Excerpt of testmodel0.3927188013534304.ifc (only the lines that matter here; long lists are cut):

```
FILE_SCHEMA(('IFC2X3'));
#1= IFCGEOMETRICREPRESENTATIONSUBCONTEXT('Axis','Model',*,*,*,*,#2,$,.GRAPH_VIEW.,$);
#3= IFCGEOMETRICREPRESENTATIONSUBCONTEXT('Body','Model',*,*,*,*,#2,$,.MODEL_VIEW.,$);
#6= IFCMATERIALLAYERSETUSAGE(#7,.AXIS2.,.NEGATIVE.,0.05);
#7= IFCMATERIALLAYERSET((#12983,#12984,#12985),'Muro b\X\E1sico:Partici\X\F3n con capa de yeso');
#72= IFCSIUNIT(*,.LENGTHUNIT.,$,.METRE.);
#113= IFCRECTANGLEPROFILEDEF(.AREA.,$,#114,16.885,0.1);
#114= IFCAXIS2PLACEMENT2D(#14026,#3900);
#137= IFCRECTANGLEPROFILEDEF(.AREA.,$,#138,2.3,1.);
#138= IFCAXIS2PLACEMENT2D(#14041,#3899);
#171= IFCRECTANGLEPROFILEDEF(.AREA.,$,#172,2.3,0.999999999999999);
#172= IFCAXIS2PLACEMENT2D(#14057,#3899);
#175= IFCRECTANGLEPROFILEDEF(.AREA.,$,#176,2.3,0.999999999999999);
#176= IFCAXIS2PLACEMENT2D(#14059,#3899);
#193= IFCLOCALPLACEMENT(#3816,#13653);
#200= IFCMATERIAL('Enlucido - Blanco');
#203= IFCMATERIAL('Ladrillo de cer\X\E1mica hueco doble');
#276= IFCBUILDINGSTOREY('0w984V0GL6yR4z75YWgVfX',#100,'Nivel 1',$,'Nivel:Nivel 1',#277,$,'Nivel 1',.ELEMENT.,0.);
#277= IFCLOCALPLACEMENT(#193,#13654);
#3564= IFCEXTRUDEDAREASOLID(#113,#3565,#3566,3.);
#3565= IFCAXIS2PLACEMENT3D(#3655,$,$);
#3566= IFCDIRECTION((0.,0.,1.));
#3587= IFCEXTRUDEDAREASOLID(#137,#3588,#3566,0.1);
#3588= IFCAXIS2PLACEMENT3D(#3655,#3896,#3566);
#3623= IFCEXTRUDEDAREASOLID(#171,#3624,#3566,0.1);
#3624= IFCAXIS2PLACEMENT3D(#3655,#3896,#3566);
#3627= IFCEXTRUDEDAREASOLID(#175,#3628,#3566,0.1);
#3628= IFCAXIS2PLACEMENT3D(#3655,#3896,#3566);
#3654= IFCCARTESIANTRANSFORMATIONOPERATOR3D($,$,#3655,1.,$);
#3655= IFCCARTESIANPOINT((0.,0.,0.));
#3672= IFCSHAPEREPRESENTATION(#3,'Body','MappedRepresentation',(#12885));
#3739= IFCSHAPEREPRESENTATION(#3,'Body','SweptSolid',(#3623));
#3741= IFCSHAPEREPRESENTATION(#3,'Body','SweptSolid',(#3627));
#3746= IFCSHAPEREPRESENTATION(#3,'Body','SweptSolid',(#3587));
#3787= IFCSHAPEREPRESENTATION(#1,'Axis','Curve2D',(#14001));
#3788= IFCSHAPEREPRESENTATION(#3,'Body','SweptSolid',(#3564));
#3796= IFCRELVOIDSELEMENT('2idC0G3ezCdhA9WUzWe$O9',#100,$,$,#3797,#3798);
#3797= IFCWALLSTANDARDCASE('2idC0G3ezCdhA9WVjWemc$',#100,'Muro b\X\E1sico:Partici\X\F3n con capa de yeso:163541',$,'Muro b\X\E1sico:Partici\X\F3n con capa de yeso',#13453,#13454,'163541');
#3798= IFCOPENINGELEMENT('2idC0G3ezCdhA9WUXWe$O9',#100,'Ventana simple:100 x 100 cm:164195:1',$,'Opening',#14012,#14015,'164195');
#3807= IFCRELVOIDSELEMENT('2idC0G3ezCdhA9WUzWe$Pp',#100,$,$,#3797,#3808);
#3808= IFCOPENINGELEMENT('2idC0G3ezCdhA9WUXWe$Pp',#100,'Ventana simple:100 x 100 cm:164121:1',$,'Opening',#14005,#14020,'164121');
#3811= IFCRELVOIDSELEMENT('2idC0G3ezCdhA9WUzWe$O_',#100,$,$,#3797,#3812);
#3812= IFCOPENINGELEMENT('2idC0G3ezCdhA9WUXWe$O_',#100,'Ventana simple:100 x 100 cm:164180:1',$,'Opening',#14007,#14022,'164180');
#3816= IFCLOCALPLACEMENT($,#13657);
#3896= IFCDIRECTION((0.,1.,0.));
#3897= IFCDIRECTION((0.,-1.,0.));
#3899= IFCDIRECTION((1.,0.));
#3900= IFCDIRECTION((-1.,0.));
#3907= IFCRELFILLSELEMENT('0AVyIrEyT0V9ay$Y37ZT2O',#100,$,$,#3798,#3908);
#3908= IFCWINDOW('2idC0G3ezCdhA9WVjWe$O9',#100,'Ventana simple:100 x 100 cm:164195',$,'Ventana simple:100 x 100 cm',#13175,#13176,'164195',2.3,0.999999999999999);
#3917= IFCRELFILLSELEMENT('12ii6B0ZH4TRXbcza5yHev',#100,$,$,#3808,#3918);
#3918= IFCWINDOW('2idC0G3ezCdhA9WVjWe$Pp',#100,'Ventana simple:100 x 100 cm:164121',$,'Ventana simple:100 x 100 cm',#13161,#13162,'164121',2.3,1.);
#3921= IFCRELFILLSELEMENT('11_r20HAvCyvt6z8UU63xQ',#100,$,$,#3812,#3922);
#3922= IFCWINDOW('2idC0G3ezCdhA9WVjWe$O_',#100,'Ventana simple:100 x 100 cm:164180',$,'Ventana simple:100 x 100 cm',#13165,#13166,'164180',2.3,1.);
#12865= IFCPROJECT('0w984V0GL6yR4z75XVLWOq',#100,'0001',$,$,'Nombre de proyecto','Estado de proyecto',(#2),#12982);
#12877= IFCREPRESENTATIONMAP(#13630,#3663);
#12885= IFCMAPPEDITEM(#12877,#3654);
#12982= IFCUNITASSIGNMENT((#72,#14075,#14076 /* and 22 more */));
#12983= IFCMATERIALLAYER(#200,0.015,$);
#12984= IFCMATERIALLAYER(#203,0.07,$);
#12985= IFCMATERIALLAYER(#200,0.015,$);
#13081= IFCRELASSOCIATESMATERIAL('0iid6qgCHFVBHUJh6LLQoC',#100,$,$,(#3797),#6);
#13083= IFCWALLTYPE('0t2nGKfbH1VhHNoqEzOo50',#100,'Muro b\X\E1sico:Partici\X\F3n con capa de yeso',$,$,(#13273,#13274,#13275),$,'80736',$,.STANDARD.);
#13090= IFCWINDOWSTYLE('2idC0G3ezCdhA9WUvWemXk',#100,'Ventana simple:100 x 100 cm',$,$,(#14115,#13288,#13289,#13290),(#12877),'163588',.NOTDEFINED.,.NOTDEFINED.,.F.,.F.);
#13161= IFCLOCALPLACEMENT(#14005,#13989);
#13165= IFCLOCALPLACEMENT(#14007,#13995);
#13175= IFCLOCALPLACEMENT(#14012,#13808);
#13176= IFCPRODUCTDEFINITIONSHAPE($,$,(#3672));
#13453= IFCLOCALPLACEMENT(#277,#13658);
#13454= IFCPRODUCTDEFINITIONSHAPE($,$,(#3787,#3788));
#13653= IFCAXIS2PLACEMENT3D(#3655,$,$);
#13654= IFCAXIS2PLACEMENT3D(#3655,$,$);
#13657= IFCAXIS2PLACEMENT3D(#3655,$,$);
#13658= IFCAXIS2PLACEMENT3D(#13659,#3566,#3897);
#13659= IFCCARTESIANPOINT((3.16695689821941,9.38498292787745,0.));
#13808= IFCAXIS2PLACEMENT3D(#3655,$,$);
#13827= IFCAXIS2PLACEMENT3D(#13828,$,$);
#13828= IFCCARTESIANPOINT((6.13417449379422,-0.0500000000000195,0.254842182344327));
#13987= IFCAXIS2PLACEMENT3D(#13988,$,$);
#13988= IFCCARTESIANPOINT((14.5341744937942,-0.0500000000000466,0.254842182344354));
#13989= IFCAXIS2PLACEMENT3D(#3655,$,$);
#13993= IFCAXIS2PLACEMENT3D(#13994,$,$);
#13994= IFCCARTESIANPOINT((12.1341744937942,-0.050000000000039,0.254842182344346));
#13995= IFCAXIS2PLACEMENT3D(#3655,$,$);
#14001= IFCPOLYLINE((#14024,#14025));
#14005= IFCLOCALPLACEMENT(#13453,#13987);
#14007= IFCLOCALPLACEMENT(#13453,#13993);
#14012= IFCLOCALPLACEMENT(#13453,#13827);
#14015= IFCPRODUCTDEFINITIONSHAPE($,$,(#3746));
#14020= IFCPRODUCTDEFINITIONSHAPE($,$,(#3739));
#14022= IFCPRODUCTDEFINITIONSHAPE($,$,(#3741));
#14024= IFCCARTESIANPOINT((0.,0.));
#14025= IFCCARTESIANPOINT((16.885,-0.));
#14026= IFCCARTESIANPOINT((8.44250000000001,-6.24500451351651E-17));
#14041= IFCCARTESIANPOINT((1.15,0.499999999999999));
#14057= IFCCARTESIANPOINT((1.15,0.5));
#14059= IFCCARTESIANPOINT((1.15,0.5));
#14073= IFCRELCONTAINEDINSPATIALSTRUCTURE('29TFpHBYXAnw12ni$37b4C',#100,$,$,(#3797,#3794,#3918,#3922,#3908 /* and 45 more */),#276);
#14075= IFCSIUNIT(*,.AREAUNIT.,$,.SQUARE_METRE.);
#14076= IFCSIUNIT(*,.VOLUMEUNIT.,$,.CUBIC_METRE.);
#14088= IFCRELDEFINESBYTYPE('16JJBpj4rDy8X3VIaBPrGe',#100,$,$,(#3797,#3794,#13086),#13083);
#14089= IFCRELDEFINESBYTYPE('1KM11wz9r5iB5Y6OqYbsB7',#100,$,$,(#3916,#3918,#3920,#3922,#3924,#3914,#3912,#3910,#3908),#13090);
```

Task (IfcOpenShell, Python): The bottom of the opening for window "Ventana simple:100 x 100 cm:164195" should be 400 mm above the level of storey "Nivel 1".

```python
import numpy as np
import ifcopenshell
import ifcopenshell.api.geometry
import ifcopenshell.geom
import ifcopenshell.util.element
import ifcopenshell.util.placement
import ifcopenshell.util.shape
import ifcopenshell.util.unit

model = ifcopenshell.open("testmodel0.3927188013534304.ifc")
unit_scale = ifcopenshell.util.unit.calculate_unit_scale(model)

window = model.by_guid("2idC0G3ezCdhA9WVjWe$O9")
opening = window.FillsVoids[0].RelatingOpeningElement
storey = ifcopenshell.util.element.get_container(window, ifc_class="IfcBuildingStorey")
level = ifcopenshell.util.placement.get_local_placement(storey.ObjectPlacement)[2, 3]

# The opening's origin need not be at the sill, so measure its lowest point.
shape = ifcopenshell.geom.create_shape(ifcopenshell.geom.settings(), opening)
bottom = ifcopenshell.util.shape.get_shape_bottom_elevation(shape, shape.geometry) / unit_scale
dz = level + 0.4 - bottom

shift = np.array([0.0, 0.0, dz])
# The window is placed relative to its opening, so it follows when the opening moves.
matrix = ifcopenshell.util.placement.get_local_placement(opening.ObjectPlacement)
matrix[:3, 3] += shift
ifcopenshell.api.geometry.edit_object_placement(
    model, product=opening, matrix=matrix, is_si=False, should_transform_children=True
)

print(f"moved by {dz * unit_scale:+.3f} m")

model.write("testmodel0.3927188013534304_updated.ifc")
```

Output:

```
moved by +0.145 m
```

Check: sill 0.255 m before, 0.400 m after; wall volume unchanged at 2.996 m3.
